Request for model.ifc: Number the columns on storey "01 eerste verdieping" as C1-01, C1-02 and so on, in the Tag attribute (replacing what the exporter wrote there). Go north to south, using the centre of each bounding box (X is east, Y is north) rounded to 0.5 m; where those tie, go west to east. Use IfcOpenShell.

First a look at what the model holds.

```python
import ifcopenshell
import ifcopenshell.util.element
import ifcopenshell.util.placement

model = ifcopenshell.open("model.ifc")
print(model.schema)
storey = next(s for s in model.by_type("IfcBuildingStorey") if s.Name == "01 eerste verdieping")
columns = [e for e in ifcopenshell.util.element.get_decomposition(storey) if e.is_a("IfcColumn")]
for e in sorted(columns, key=lambda e: e.id()):
    origin = ifcopenshell.util.placement.get_local_placement(e.ObjectPlacement)[:3, 3]
    print(e.id(), e.Tag, e.Name, origin.round(2) + 0.0, sep=" | ")
```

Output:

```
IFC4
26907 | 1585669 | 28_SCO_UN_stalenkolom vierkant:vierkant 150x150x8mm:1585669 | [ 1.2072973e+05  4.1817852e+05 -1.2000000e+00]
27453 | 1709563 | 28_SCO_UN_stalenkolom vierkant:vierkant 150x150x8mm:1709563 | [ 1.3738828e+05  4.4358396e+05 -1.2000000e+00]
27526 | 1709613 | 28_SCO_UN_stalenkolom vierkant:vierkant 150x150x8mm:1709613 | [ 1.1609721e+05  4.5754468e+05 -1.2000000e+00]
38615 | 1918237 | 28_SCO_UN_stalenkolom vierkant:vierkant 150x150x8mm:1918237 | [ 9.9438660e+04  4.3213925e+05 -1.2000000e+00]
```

```python
import ifcopenshell
import ifcopenshell.geom
import ifcopenshell.util.element
import ifcopenshell.util.shape

model = ifcopenshell.open("model.ifc")
settings = ifcopenshell.geom.settings()
settings.set("use-world-coords", True)


def centre(element):
    shape = ifcopenshell.geom.create_shape(settings, element)
    return ifcopenshell.util.shape.get_bbox_centroid(shape.geometry)


storey = next(s for s in model.by_type("IfcBuildingStorey") if s.Name == "01 eerste verdieping")
columns = [e for e in ifcopenshell.util.element.get_decomposition(storey) if e.is_a("IfcColumn")]

# Insertion points can sit at a corner or the storey origin, so sort by the geometry (in metres).
centres = {e: centre(e) for e in columns}
columns.sort(key=lambda e: (-round(centres[e][1] / 0.5), centres[e][0]))

for i, e in enumerate(columns, start=1):
    number = f"C1-{i:02d}"
    e.Tag = number
    print(e.id(), number)

model.write("model_v2.ifc")
```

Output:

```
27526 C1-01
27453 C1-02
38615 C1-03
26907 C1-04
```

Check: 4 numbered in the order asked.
